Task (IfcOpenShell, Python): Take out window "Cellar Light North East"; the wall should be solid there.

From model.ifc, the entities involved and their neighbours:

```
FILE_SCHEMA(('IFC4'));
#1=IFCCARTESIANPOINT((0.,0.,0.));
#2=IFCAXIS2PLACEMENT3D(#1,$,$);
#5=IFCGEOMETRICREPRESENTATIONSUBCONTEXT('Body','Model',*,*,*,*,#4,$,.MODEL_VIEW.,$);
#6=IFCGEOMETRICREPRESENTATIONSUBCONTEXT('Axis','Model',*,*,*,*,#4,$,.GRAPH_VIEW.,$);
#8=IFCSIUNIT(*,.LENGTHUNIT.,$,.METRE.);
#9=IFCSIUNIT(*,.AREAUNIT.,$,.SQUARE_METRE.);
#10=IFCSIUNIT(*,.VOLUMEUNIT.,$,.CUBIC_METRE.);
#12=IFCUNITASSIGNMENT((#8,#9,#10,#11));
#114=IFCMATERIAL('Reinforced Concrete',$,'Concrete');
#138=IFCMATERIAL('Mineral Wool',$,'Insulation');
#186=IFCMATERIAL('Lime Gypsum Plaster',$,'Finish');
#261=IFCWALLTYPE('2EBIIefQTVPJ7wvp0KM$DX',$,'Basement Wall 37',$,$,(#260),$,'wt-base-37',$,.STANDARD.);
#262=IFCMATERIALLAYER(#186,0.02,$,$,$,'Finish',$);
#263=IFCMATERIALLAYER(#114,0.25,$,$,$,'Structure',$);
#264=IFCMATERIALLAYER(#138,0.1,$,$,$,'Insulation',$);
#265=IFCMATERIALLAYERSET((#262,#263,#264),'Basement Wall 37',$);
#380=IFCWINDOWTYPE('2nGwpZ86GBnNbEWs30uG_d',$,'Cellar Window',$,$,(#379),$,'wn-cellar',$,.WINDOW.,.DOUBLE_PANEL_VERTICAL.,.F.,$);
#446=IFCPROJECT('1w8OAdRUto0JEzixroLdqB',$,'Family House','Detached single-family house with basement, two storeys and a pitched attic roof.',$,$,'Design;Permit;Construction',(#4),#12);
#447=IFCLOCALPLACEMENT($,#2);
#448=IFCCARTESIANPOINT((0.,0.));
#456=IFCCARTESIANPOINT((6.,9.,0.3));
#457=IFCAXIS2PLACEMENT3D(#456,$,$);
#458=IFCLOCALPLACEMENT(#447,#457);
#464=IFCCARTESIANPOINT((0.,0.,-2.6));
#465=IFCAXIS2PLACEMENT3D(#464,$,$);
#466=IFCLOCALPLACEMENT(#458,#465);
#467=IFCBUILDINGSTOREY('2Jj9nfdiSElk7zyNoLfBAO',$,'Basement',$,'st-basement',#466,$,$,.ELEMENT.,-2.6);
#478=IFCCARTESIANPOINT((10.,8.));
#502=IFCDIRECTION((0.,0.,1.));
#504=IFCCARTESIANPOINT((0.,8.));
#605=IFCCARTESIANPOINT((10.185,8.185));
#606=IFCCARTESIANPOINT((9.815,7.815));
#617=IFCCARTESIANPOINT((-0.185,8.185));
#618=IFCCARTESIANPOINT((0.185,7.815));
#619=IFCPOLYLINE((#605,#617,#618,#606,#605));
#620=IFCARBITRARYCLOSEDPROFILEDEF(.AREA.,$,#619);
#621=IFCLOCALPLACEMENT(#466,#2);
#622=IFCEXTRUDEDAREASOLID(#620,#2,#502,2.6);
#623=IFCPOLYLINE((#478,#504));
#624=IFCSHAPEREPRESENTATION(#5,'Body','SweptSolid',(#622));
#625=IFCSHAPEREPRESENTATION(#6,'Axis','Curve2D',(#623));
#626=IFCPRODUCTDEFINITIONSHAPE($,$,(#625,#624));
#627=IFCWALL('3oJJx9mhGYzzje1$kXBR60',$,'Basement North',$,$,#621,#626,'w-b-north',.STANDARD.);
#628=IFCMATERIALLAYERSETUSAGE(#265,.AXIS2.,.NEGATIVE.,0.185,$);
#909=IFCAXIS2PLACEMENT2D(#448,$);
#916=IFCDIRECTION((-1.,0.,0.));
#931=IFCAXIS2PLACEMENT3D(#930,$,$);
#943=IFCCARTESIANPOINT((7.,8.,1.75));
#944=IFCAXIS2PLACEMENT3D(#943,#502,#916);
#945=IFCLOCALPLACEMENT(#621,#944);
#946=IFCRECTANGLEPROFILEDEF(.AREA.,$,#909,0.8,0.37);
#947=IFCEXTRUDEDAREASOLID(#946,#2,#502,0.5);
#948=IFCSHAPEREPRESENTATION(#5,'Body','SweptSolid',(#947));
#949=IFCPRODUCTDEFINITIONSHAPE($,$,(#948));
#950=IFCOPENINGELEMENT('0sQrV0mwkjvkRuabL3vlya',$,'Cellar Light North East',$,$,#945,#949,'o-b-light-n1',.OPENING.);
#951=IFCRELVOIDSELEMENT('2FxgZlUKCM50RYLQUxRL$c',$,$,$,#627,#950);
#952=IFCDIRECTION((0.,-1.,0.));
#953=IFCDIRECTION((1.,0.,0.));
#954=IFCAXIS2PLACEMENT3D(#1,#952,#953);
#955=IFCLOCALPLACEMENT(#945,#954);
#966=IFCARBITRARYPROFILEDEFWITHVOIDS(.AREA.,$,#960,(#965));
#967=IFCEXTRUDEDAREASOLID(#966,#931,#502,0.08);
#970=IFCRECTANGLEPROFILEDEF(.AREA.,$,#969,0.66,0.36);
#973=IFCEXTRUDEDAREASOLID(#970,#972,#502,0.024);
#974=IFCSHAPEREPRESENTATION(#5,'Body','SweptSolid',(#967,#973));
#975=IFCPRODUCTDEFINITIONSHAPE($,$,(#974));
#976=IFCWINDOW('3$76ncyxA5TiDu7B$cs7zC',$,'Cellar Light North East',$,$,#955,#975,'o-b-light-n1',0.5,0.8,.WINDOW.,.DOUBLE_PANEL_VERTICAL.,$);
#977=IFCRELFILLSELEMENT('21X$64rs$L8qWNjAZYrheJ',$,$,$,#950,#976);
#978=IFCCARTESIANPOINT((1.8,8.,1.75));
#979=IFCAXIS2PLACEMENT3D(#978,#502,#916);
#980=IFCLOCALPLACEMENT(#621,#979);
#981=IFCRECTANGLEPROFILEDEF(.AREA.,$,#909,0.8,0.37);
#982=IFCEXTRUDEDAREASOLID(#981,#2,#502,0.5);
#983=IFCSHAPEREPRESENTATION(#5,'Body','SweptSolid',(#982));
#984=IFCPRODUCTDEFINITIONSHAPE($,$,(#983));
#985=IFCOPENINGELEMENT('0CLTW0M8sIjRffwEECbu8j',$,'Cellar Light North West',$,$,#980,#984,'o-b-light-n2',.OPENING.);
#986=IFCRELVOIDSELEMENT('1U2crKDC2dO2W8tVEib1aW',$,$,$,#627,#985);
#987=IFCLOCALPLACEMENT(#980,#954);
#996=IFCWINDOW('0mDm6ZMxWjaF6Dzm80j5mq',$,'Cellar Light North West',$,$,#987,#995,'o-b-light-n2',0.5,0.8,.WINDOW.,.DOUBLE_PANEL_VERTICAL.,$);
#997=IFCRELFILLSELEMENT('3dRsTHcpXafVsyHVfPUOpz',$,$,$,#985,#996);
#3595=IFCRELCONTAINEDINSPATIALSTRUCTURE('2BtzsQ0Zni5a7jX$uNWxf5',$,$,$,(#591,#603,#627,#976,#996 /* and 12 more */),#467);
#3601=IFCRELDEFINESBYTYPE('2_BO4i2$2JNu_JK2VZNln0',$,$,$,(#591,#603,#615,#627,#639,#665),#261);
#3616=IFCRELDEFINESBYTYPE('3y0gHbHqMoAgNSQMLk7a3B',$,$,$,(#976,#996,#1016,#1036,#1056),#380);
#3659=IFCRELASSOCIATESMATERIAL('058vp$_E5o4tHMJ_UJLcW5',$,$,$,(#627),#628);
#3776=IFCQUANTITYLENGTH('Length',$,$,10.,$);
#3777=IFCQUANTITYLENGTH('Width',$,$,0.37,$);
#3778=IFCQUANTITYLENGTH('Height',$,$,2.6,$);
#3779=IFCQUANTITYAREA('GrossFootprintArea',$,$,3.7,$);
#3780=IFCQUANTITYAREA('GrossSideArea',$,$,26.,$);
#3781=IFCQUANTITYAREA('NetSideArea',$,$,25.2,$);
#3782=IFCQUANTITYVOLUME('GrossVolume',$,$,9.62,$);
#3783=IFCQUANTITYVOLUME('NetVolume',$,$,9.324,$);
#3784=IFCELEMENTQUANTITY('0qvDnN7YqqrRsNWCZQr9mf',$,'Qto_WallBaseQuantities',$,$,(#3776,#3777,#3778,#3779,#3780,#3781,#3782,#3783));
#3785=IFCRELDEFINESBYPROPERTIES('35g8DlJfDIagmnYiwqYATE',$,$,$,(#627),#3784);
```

```python
import ifcopenshell
import ifcopenshell.api.feature
import ifcopenshell.api.pset
import ifcopenshell.api.root
import ifcopenshell.geom
import ifcopenshell.util.element
import ifcopenshell.util.shape
import ifcopenshell.util.unit

model = ifcopenshell.open("model.ifc")
area_scale = ifcopenshell.util.unit.calculate_unit_scale(model, "AREAUNIT")
volume_scale = ifcopenshell.util.unit.calculate_unit_scale(model, "VOLUMEUNIT")
settings = ifcopenshell.geom.settings()


def volume(element):
    """Net volume in cubic metres, openings subtracted."""
    shape = ifcopenshell.geom.create_shape(settings, element)
    return ifcopenshell.util.shape.get_volume(shape.geometry)


window = model.by_guid("3$76ncyxA5TiDu7B$cs7zC")
opening = window.FillsVoids[0].RelatingOpeningElement
wall = opening.VoidsElements[0].RelatingBuildingElement
before = volume(wall)

ifcopenshell.api.root.remove_product(model, product=window)
ifcopenshell.api.feature.remove_feature(model, feature=opening)

after = volume(wall)
thickness = 0.37  # wall thickness in metres

# Update the wall's stored quantities.
qto = model.by_id(ifcopenshell.util.element.get_pset(wall, "Qto_WallBaseQuantities", should_inherit=False)["id"])
ifcopenshell.api.pset.edit_qto(model, qto=qto, properties={
    "NetSideArea": after / thickness / area_scale,
    "NetVolume": after / volume_scale,
})

print(f"wall volume {before:.3f} -> {after:.3f} m3")

model.write("model_updated.ifc")
```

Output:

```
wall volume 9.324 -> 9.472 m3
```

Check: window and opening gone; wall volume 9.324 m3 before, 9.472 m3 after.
